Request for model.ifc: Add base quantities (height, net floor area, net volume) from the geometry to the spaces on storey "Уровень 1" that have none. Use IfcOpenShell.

First a look at what the model holds.

```python
import ifcopenshell
import ifcopenshell.util.element
import ifcopenshell.util.unit

model = ifcopenshell.open("model.ifc")
print(model.schema)
for unit_type in ("LENGTHUNIT", "AREAUNIT", "VOLUMEUNIT"):
    print(unit_type, ifcopenshell.util.unit.calculate_unit_scale(model, unit_type))
storey = next(s for s in model.by_type("IfcBuildingStorey") if s.Name == "Уровень 1")
spaces = [e for e in ifcopenshell.util.element.get_decomposition(storey) if e.is_a("IfcSpace")]
for e in sorted(spaces, key=lambda e: e.id()):
    print(e.id(), e.is_a(), e.Name, list(ifcopenshell.util.element.get_psets(e, qtos_only=True)), sep=" | ")
```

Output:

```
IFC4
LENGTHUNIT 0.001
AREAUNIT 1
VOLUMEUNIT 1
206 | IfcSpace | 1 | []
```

```python
import ifcopenshell
import ifcopenshell.api.pset
import ifcopenshell.geom
import ifcopenshell.util.element
import ifcopenshell.util.shape
import ifcopenshell.util.unit

model = ifcopenshell.open("model.ifc")
unit_scale = ifcopenshell.util.unit.calculate_unit_scale(model)
area_scale = ifcopenshell.util.unit.calculate_unit_scale(model, "AREAUNIT")
volume_scale = ifcopenshell.util.unit.calculate_unit_scale(model, "VOLUMEUNIT")
settings = ifcopenshell.geom.settings()

storey = next(s for s in model.by_type("IfcBuildingStorey") if s.Name == "Уровень 1")
spaces = [e for e in ifcopenshell.util.element.get_decomposition(storey) if e.is_a("IfcSpace")]

for e in sorted(spaces, key=lambda e: e.id()):
    if ifcopenshell.util.element.get_psets(e, qtos_only=True, should_inherit=False):
        continue
    # Geometry comes back in metres, in the element's own axes.
    shape = ifcopenshell.geom.create_shape(settings, e)
    values = {
        "Height": ifcopenshell.util.shape.get_z(shape.geometry) / unit_scale,
        "NetFloorArea": ifcopenshell.util.shape.get_footprint_area(shape.geometry) / area_scale,
        "NetVolume": ifcopenshell.util.shape.get_volume(shape.geometry) / volume_scale,
    }
    qto = ifcopenshell.api.pset.add_qto(model, product=e, name="Qto_SpaceBaseQuantities")
    ifcopenshell.api.pset.edit_qto(model, qto=qto, properties=values)
    print(e.id(), {k: round(v, 3) for k, v in values.items()})

model.write("model_rev.ifc")
```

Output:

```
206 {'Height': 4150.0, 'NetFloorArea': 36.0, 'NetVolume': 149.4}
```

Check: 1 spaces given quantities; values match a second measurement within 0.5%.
